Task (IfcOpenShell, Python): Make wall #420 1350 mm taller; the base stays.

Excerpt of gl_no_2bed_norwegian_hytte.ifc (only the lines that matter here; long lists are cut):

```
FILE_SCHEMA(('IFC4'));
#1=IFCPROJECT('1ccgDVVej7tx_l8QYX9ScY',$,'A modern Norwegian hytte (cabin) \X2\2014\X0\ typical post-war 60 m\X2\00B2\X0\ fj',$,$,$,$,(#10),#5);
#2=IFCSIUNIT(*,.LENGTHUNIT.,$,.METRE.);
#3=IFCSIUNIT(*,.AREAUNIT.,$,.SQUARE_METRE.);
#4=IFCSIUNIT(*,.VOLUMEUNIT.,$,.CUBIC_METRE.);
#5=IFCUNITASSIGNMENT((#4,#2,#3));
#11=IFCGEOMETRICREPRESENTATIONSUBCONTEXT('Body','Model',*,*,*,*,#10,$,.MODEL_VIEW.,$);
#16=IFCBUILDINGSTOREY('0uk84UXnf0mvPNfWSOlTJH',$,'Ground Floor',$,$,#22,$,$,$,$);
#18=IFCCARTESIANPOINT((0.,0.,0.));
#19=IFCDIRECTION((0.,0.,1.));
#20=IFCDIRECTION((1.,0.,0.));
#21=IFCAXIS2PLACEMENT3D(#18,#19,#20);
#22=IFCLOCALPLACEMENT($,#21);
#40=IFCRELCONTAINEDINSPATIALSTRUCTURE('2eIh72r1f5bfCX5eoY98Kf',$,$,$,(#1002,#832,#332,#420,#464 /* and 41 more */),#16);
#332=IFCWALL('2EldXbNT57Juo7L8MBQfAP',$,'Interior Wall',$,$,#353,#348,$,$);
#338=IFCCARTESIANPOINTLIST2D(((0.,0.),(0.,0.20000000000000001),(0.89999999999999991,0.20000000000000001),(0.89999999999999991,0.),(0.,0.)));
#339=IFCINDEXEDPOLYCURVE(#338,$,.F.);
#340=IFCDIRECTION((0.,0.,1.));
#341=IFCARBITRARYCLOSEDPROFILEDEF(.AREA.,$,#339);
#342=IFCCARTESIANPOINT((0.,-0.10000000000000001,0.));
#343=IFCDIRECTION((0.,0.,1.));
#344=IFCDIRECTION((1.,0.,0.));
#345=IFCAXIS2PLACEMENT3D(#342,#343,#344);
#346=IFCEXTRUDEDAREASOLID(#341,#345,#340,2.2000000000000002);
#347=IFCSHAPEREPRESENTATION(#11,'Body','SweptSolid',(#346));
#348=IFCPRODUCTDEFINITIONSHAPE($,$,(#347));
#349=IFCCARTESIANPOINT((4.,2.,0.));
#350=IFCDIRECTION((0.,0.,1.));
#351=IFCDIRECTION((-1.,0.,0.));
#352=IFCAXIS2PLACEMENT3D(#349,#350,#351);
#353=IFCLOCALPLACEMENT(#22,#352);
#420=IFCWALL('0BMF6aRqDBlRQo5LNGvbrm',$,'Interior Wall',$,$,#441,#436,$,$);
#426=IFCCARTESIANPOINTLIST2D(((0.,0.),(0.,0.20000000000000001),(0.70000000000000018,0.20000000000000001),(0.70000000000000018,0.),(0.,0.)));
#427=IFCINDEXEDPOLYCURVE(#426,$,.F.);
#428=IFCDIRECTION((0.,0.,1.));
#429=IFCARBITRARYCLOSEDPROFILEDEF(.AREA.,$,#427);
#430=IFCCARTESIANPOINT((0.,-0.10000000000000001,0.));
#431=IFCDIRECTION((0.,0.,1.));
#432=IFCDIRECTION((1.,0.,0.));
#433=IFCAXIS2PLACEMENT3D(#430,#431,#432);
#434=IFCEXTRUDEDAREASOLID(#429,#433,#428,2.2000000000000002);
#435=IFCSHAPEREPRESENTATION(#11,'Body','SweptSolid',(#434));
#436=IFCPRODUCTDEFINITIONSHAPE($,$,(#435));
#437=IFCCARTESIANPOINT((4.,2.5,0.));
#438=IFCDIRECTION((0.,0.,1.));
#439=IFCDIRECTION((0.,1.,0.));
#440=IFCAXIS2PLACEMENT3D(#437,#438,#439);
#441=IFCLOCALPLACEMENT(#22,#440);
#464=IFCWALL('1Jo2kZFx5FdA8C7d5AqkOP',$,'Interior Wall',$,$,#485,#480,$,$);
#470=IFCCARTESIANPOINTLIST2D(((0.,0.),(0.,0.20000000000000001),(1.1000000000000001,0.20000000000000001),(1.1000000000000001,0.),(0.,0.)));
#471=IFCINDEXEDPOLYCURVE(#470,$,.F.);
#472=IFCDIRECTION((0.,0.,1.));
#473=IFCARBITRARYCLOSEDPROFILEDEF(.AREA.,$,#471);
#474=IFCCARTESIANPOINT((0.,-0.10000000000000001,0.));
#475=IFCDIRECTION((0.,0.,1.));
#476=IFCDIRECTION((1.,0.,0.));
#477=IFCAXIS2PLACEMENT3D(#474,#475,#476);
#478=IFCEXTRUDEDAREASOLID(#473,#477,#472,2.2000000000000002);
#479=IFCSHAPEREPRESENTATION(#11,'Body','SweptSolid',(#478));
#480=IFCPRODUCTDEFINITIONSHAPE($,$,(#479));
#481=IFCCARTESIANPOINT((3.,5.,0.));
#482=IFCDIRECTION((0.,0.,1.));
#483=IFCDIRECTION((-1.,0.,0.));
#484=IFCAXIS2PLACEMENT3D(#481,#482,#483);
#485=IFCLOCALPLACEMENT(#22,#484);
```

```python
import ifcopenshell
import ifcopenshell.geom
import ifcopenshell.util.representation
import ifcopenshell.util.shape

model = ifcopenshell.open("gl_no_2bed_norwegian_hytte.ifc")
settings = ifcopenshell.geom.settings()


def volume(element):
    """Net volume in cubic metres, openings subtracted."""
    shape = ifcopenshell.geom.create_shape(settings, element)
    return ifcopenshell.util.shape.get_volume(shape.geometry)


wall = model.by_id(420)
before = volume(wall)

body = ifcopenshell.util.representation.get_representation(wall, "Model", "Body")
solid = body.Items[0]
old_height = solid.Depth
solid.Depth += 1.35
after = volume(wall)

print(f"height {old_height:g} -> {solid.Depth:g}, volume {before:.3f} -> {after:.3f} m3")

model.write("gl_no_2bed_norwegian_hytte_rev.ifc")
```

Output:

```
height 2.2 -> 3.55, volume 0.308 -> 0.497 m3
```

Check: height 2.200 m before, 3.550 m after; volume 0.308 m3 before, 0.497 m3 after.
